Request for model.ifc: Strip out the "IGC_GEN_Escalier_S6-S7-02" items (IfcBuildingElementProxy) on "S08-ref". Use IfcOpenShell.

First a look at what the model holds.

```python
import ifcopenshell
import ifcopenshell.util.element

model = ifcopenshell.open("model.ifc")
print(model.schema)
storey = next(s for s in model.by_type("IfcBuildingStorey") if s.Name == "S08-ref")
proxies = [e for e in ifcopenshell.util.element.get_decomposition(storey) if e.is_a("IfcBuildingElementProxy")]
seen = {}
for e in proxies:
    element_type = ifcopenshell.util.element.get_type(e)
    name = element_type.Name if element_type not in (None, e) else None
    seen[name] = seen.get(name, 0) + 1
for name, count in sorted(seen.items(), key=str):
    print(count, "x", name)
```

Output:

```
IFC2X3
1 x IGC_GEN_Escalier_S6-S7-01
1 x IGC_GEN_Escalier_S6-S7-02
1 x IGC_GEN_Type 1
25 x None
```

```python
import ifcopenshell
import ifcopenshell.api.root
import ifcopenshell.util.element

model = ifcopenshell.open("model.ifc")

storey = next(s for s in model.by_type("IfcBuildingStorey") if s.Name == "S08-ref")
proxies = [e for e in ifcopenshell.util.element.get_decomposition(storey) if e.is_a("IfcBuildingElementProxy")]
targets = [e for e in proxies if (t := ifcopenshell.util.element.get_type(e)) not in (None, e) and t.Name == "IGC_GEN_Escalier_S6-S7-02"]

for e in targets:
    ifcopenshell.api.root.remove_product(model, product=e)
print(len(targets), "removed")

model.write("model_edited.ifc")
```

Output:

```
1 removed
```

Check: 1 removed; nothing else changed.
